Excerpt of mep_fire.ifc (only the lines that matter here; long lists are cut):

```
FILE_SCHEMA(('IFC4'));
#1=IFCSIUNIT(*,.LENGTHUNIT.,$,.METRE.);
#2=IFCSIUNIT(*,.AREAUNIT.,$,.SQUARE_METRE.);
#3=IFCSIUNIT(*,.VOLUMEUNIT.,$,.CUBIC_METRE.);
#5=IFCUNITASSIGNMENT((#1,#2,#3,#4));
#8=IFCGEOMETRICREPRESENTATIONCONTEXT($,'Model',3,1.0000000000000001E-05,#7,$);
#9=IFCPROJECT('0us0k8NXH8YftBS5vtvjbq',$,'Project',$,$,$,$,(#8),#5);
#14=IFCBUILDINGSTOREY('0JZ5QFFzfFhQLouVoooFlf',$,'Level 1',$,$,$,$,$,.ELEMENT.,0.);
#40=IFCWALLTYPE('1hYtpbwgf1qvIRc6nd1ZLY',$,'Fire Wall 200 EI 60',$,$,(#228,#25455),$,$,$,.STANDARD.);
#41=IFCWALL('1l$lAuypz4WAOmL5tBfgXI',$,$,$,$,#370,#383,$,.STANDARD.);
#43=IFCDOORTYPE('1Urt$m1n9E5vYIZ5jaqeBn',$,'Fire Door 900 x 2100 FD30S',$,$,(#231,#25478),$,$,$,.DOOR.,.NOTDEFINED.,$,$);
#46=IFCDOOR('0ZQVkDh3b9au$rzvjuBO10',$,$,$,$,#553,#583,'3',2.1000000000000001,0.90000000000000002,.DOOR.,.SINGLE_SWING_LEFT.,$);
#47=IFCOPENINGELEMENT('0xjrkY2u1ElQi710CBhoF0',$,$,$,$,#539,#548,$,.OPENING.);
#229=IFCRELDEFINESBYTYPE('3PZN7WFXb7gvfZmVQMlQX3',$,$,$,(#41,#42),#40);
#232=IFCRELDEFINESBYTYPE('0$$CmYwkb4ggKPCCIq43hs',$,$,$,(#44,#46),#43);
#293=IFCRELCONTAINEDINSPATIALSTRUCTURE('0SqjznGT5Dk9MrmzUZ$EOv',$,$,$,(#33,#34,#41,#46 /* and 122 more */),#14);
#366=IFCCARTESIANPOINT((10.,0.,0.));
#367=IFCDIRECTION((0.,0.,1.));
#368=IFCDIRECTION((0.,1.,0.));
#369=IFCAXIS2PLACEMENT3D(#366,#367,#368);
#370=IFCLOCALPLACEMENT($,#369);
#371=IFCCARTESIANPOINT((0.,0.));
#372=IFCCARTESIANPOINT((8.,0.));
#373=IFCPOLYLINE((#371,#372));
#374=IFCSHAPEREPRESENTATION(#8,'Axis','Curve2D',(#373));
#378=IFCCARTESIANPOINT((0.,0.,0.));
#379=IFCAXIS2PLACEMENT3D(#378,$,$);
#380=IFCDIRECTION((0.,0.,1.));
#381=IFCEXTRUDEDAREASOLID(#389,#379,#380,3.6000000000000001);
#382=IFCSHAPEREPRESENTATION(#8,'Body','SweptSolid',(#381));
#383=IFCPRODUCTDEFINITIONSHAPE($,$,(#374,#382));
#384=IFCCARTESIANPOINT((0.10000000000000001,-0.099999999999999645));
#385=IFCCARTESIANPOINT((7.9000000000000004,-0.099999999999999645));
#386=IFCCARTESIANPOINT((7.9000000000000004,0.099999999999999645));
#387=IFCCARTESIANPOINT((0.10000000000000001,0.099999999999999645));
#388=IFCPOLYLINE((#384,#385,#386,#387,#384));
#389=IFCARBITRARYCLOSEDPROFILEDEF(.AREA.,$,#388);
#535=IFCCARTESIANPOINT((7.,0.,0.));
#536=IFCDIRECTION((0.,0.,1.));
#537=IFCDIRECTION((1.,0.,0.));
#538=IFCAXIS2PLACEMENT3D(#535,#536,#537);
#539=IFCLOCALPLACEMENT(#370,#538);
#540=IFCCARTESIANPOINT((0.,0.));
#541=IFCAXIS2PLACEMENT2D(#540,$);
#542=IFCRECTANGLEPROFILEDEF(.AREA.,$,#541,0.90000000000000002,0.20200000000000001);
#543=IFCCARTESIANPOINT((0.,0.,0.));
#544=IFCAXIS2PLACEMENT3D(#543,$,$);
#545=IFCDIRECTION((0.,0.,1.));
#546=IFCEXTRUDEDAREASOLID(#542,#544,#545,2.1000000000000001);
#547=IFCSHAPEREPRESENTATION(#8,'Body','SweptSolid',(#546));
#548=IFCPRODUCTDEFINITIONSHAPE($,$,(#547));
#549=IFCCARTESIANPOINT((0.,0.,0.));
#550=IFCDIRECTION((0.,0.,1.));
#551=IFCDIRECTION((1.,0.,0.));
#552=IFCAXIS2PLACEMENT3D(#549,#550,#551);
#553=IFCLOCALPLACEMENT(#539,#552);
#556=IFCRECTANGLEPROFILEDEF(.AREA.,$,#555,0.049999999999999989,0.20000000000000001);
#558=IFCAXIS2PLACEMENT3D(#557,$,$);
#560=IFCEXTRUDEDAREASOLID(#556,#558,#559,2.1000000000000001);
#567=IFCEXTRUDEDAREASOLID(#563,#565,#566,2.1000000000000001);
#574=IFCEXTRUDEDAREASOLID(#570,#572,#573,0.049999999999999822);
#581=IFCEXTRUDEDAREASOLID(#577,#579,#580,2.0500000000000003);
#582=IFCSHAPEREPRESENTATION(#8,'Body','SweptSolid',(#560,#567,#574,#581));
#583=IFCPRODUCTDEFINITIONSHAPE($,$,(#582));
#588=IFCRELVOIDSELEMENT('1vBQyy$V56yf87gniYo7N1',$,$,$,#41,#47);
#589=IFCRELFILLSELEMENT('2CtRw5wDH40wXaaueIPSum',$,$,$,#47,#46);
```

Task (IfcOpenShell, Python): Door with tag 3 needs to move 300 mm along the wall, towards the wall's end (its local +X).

```python
import ifcopenshell
import ifcopenshell.api.geometry
import ifcopenshell.util.placement
import ifcopenshell.util.unit

model = ifcopenshell.open("mep_fire.ifc")
unit_scale = ifcopenshell.util.unit.calculate_unit_scale(model)

door = model.by_id(46)
opening = door.FillsVoids[0].RelatingOpeningElement
wall = opening.VoidsElements[0].RelatingBuildingElement

wall_matrix = ifcopenshell.util.placement.get_local_placement(wall.ObjectPlacement)
shift = wall_matrix[:3, 0] * 0.3 / unit_scale
before = ifcopenshell.util.placement.get_local_placement(door.ObjectPlacement)[:3, 3].copy()

# The door is placed relative to its opening, so it follows when the opening moves.
matrix = ifcopenshell.util.placement.get_local_placement(opening.ObjectPlacement)
matrix[:3, 3] += shift
ifcopenshell.api.geometry.edit_object_placement(
    model, product=opening, matrix=matrix, is_si=False, should_transform_children=True
)

after = ifcopenshell.util.placement.get_local_placement(door.ObjectPlacement)[:3, 3]
print("door moved by", (after - before).round(3) + 0.0)

model.write("mep_fire_edited.ifc")
```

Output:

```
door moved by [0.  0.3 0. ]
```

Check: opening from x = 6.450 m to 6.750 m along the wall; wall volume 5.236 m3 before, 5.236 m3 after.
